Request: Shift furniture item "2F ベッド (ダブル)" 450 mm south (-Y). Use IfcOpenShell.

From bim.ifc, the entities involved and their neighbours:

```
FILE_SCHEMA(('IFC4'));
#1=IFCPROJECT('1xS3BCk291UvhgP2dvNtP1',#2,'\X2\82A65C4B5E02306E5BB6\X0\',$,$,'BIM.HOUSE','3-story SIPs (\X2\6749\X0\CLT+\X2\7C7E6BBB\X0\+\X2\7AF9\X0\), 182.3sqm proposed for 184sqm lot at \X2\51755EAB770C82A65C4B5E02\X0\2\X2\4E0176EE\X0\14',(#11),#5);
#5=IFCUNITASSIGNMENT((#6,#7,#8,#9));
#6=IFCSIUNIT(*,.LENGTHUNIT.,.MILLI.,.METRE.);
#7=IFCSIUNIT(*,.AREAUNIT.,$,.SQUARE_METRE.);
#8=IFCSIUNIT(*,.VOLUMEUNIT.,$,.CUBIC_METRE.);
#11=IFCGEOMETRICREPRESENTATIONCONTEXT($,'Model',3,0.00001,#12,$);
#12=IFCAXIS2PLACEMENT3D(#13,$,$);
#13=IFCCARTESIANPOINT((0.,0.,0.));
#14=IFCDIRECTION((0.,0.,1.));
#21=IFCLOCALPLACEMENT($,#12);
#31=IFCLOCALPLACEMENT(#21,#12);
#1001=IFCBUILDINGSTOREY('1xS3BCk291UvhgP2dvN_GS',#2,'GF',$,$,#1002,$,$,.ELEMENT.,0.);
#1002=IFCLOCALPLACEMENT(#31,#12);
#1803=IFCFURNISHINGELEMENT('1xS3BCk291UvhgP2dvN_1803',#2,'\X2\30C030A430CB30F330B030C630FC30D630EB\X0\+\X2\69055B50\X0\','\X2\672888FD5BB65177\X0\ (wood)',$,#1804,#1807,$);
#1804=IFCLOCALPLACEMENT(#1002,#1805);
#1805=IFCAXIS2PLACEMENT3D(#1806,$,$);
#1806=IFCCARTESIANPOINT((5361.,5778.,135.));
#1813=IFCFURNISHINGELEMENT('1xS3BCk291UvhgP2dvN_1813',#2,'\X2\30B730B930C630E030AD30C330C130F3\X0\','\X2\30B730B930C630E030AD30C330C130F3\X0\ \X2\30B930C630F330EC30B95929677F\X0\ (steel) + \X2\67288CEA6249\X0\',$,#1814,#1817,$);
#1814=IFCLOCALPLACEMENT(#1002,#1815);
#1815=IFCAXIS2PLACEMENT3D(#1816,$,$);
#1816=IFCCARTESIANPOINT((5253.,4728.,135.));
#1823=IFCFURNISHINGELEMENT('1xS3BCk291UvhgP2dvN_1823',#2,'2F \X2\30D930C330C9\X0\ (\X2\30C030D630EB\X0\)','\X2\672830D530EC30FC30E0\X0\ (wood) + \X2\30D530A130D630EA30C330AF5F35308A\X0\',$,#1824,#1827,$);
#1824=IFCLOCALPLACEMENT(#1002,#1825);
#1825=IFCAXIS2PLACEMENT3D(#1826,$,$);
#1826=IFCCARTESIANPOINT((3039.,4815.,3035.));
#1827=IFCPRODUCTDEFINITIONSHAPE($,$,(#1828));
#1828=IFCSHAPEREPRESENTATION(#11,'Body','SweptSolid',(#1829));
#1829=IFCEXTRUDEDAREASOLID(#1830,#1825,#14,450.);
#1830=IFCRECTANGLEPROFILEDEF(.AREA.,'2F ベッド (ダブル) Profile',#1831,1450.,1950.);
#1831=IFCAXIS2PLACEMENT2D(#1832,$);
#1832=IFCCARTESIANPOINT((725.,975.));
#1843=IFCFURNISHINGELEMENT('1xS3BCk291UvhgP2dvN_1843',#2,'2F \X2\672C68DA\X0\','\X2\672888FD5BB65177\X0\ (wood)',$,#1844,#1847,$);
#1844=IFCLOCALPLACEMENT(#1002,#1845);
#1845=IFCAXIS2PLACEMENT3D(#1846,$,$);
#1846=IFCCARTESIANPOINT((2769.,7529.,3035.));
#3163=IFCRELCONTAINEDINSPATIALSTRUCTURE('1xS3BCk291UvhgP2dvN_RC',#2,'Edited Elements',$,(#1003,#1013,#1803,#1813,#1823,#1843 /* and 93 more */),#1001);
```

```python
import ifcopenshell
import ifcopenshell.api.geometry
import ifcopenshell.util.placement

model = ifcopenshell.open("bim.ifc")

item = model.by_guid("1xS3BCk291UvhgP2dvN_1823")
matrix = ifcopenshell.util.placement.get_local_placement(item.ObjectPlacement)
matrix[1, 3] -= 450.0
ifcopenshell.api.geometry.edit_object_placement(model, product=item, matrix=matrix, is_si=False)

print(ifcopenshell.util.placement.get_local_placement(item.ObjectPlacement).round(3) + 0.0)

model.write("bim_v2.ifc")
```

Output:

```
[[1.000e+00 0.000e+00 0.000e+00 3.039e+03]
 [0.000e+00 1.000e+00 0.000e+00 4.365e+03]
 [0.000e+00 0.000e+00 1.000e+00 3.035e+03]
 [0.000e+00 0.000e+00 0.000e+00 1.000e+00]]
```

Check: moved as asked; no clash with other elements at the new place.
